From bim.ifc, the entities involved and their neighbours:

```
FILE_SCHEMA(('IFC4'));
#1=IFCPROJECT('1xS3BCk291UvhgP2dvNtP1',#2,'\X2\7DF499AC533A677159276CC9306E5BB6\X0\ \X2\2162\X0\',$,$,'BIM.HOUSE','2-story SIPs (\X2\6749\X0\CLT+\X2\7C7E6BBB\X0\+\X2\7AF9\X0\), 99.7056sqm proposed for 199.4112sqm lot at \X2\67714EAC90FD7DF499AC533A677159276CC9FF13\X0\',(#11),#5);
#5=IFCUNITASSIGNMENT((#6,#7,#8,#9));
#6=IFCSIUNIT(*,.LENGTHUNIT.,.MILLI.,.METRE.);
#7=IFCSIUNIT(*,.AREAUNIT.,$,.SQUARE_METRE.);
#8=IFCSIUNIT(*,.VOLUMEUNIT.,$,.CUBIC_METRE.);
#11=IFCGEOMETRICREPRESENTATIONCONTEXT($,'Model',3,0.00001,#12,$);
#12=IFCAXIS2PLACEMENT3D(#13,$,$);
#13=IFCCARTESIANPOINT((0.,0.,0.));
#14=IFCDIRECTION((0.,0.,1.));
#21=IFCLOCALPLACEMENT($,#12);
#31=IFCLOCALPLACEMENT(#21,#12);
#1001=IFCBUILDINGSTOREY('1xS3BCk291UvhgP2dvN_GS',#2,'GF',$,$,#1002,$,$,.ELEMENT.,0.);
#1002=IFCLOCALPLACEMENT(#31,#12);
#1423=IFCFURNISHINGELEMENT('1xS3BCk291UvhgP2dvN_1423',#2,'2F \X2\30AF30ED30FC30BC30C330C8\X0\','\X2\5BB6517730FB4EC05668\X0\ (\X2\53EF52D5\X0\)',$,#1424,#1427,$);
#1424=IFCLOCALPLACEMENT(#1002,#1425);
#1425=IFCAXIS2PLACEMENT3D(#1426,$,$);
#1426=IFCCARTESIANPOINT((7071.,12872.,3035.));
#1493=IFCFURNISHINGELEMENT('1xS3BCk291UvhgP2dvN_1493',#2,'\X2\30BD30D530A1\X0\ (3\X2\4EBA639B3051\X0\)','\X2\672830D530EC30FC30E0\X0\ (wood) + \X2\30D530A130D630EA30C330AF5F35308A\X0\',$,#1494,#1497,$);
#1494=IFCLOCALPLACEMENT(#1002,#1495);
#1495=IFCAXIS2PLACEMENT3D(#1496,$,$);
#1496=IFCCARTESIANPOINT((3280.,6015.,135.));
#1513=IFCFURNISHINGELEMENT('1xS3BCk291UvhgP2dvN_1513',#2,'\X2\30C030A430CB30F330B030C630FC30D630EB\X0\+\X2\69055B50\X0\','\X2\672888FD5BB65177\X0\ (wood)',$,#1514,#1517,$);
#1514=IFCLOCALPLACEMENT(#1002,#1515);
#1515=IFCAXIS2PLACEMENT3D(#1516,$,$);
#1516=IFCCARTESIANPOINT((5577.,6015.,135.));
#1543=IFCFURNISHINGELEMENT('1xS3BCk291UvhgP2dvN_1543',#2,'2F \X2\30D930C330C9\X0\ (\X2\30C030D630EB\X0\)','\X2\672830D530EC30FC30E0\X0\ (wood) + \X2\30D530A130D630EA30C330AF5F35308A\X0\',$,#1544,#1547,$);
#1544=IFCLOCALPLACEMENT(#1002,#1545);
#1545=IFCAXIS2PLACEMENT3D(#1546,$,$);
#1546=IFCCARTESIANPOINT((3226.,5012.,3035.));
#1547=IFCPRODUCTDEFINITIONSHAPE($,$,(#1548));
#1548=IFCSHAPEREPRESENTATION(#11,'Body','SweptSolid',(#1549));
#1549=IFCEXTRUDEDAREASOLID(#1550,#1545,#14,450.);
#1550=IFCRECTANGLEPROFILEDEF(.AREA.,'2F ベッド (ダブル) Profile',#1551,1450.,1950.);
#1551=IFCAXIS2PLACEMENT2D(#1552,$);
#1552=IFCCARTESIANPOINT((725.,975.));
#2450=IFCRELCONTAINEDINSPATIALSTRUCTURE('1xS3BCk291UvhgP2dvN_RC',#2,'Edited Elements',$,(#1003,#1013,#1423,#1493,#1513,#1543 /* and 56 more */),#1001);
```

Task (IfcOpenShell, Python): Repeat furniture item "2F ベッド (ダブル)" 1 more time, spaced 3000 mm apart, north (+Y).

```python
import numpy as np
import ifcopenshell
import ifcopenshell.api.geometry
import ifcopenshell.api.root
import ifcopenshell.util.element
import ifcopenshell.util.placement
import ifcopenshell.util.unit

model = ifcopenshell.open("bim.ifc")
unit_scale = ifcopenshell.util.unit.calculate_unit_scale(model)


def reuse_history(source, copy):
    """copy_class also copies each property set's owner history, people and application; keep the originals."""
    for rel in copy.IsDefinedBy:
        if rel.is_a("IfcRelDefinesByProperties") and (history := rel.RelatingPropertyDefinition.OwnerHistory):
            rel.RelatingPropertyDefinition.OwnerHistory = source.OwnerHistory
            ifcopenshell.util.element.remove_deep2(model, history)


source = model.by_guid("1xS3BCk291UvhgP2dvN_1543")
base = ifcopenshell.util.placement.get_local_placement(source.ObjectPlacement)
step = np.array([0.0, 1.0, 0.0]) * 3 / unit_scale

for i in range(1, 2):
    copy = ifcopenshell.api.root.copy_class(model, product=source)
    copy.Representation = ifcopenshell.util.element.copy_deep(
        model, source.Representation, exclude=["IfcGeometricRepresentationContext", "IfcRepresentationMap"]
    )
    reuse_history(source, copy)
    matrix = base.copy()
    matrix[:3, 3] += i * step
    print("added at", matrix[:3, 3].round(3) + 0.0)
    ifcopenshell.api.geometry.edit_object_placement(model, product=copy, matrix=matrix, is_si=False)

model.write("bim-out.ifc")
```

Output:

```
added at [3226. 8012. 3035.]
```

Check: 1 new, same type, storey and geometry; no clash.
